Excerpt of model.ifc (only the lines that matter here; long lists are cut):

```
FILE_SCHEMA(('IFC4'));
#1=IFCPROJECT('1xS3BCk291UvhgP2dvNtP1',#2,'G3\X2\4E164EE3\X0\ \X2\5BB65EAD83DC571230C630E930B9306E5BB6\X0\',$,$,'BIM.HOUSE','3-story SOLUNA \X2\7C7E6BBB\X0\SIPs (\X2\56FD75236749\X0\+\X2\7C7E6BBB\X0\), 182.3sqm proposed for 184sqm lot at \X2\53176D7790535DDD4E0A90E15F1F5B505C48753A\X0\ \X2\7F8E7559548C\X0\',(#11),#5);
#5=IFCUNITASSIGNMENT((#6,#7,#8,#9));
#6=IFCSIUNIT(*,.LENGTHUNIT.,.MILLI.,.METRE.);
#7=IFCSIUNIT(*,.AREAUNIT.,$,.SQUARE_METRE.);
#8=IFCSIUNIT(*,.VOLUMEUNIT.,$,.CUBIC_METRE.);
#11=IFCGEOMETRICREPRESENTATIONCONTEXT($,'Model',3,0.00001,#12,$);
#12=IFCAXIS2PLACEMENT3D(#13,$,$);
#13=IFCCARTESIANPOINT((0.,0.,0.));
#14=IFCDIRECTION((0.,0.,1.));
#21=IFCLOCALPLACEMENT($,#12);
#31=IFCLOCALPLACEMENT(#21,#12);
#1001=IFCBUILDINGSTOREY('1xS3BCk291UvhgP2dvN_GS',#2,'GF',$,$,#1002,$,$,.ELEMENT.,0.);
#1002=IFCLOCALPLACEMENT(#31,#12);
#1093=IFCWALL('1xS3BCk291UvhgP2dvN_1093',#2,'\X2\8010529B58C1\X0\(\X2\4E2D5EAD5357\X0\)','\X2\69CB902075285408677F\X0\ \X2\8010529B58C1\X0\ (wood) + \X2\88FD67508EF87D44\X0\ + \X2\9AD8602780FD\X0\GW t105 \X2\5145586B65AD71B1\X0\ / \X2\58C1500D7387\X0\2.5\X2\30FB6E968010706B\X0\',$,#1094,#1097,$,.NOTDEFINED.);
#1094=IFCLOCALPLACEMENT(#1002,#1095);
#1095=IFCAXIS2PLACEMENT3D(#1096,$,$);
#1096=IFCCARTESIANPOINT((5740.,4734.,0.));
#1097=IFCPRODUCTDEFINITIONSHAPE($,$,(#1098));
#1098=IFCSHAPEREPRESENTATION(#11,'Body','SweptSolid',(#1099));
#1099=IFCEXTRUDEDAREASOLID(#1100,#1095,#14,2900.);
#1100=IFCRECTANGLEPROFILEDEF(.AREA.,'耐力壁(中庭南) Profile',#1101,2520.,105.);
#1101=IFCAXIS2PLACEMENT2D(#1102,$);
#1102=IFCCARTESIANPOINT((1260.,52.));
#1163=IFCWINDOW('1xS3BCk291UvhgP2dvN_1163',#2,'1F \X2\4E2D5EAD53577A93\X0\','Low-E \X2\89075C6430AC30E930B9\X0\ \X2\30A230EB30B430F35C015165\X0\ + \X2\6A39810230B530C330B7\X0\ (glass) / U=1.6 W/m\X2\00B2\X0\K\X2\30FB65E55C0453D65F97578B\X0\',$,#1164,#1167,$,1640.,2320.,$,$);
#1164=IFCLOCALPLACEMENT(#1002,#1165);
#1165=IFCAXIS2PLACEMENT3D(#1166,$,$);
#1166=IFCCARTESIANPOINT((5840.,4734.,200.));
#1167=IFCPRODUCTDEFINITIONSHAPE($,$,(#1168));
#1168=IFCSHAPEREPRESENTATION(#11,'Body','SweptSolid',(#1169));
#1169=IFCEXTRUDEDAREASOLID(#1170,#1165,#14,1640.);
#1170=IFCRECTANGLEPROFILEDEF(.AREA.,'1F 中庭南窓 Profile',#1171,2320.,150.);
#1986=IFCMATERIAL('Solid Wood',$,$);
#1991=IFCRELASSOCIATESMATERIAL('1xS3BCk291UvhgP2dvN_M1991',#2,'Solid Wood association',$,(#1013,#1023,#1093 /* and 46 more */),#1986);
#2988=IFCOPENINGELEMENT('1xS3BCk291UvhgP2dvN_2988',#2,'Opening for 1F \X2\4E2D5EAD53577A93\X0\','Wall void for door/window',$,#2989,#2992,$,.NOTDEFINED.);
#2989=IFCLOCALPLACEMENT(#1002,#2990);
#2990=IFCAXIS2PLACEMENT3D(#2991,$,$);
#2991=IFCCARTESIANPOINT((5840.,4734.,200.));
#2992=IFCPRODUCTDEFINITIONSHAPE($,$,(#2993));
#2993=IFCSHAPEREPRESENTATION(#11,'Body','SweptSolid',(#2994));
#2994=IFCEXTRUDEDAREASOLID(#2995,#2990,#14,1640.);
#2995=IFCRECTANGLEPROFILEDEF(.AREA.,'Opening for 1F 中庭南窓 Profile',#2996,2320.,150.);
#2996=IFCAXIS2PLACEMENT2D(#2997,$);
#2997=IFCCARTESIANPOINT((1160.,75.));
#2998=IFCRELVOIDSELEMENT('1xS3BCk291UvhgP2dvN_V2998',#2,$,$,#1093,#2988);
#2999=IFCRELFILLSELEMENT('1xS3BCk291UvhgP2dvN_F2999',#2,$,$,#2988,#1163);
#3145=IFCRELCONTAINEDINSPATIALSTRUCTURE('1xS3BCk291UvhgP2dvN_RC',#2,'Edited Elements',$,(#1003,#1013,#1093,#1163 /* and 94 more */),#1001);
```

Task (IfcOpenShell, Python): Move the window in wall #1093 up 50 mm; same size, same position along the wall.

```python
import numpy as np
import ifcopenshell
import ifcopenshell.api.geometry
import ifcopenshell.util.placement
import ifcopenshell.util.unit

model = ifcopenshell.open("model.ifc")
unit_scale = ifcopenshell.util.unit.calculate_unit_scale(model)

window = model.by_guid("1xS3BCk291UvhgP2dvN_1163")
opening = window.FillsVoids[0].RelatingOpeningElement
dz = 0.05 / unit_scale

shift = np.array([0.0, 0.0, dz])
# The window is not placed relative to its opening, so move both.
for product in (opening, window):
    matrix = ifcopenshell.util.placement.get_local_placement(product.ObjectPlacement)
    matrix[:3, 3] += shift
    ifcopenshell.api.geometry.edit_object_placement(model, product=product, matrix=matrix, is_si=False)

print(f"moved by {dz * unit_scale:+.3f} m")

model.write("model_v2.ifc")
```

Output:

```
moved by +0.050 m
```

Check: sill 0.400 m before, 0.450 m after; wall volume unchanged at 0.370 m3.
